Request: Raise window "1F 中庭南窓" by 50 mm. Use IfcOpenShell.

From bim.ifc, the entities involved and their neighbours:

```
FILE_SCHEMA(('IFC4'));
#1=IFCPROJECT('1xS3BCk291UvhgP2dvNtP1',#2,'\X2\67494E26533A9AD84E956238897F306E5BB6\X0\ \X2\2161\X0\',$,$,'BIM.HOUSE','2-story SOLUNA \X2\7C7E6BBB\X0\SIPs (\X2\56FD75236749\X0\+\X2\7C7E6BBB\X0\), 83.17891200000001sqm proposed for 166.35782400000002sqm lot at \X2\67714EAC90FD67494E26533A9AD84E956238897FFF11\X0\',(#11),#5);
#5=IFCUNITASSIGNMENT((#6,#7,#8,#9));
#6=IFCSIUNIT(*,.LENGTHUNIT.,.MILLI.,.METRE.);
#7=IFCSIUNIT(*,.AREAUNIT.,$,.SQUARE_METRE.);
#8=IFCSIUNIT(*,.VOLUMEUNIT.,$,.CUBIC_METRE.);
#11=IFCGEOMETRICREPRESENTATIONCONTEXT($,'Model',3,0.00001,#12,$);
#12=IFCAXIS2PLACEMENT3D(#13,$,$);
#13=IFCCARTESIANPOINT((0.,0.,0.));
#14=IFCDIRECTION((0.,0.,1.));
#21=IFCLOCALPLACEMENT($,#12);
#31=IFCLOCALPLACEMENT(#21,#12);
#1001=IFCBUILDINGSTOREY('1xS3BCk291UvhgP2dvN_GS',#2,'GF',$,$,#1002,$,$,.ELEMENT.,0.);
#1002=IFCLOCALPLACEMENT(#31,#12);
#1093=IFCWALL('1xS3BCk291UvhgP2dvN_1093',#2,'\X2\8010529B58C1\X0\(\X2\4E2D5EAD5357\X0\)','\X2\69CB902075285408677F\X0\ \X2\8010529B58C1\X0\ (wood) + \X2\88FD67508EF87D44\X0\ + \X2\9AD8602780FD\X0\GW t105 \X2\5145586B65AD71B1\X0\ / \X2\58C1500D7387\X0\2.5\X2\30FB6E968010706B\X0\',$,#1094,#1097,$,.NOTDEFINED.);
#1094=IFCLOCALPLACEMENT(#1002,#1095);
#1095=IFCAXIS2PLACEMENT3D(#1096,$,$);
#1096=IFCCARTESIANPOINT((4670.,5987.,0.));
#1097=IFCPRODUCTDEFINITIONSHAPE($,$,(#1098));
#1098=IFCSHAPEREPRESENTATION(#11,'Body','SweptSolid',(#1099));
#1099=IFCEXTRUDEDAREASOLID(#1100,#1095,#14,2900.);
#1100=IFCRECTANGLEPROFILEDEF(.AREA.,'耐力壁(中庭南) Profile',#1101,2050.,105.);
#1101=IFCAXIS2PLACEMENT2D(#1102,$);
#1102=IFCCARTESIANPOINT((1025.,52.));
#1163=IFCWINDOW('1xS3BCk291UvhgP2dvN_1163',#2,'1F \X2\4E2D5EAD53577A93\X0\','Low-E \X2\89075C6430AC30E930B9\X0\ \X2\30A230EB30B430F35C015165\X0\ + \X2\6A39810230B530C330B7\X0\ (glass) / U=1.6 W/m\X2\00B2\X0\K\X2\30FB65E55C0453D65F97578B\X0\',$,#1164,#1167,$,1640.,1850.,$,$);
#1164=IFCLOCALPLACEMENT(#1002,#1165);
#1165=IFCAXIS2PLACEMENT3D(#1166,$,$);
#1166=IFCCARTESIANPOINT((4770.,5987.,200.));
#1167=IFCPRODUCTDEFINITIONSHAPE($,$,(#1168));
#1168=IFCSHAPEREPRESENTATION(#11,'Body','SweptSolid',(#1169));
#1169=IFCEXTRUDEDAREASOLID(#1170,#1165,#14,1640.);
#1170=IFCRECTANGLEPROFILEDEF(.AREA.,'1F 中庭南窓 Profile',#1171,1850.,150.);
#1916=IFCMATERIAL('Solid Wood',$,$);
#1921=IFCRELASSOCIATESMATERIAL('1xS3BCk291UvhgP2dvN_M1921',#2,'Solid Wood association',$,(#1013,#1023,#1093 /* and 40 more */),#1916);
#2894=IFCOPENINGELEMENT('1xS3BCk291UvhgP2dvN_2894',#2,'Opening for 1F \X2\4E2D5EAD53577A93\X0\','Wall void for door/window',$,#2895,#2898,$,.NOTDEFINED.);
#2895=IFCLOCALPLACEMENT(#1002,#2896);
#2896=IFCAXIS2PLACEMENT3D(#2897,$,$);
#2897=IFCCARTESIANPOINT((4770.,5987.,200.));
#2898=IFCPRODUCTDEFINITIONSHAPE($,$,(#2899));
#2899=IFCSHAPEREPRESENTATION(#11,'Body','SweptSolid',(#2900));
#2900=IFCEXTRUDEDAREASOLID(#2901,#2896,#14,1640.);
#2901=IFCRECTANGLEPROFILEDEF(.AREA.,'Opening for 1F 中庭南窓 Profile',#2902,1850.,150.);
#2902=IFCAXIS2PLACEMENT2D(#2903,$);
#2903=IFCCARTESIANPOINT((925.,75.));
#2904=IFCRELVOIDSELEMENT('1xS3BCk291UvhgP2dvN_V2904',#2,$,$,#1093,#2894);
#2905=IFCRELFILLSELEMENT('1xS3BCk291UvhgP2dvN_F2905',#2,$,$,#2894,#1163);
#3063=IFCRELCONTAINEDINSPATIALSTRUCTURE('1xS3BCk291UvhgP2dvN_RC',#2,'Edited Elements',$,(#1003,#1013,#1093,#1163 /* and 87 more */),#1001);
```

```python
import numpy as np
import ifcopenshell
import ifcopenshell.api.geometry
import ifcopenshell.util.placement
import ifcopenshell.util.unit

model = ifcopenshell.open("bim.ifc")
unit_scale = ifcopenshell.util.unit.calculate_unit_scale(model)

window = model.by_guid("1xS3BCk291UvhgP2dvN_1163")
opening = window.FillsVoids[0].RelatingOpeningElement
dz = 0.05 / unit_scale

shift = np.array([0.0, 0.0, dz])
# The window is not placed relative to its opening, so move both.
for product in (opening, window):
    matrix = ifcopenshell.util.placement.get_local_placement(product.ObjectPlacement)
    matrix[:3, 3] += shift
    ifcopenshell.api.geometry.edit_object_placement(model, product=product, matrix=matrix, is_si=False)

print(f"moved by {dz * unit_scale:+.3f} m")

model.write("bim_v2.ifc")
```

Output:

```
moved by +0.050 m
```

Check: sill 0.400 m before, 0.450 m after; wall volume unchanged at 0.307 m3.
